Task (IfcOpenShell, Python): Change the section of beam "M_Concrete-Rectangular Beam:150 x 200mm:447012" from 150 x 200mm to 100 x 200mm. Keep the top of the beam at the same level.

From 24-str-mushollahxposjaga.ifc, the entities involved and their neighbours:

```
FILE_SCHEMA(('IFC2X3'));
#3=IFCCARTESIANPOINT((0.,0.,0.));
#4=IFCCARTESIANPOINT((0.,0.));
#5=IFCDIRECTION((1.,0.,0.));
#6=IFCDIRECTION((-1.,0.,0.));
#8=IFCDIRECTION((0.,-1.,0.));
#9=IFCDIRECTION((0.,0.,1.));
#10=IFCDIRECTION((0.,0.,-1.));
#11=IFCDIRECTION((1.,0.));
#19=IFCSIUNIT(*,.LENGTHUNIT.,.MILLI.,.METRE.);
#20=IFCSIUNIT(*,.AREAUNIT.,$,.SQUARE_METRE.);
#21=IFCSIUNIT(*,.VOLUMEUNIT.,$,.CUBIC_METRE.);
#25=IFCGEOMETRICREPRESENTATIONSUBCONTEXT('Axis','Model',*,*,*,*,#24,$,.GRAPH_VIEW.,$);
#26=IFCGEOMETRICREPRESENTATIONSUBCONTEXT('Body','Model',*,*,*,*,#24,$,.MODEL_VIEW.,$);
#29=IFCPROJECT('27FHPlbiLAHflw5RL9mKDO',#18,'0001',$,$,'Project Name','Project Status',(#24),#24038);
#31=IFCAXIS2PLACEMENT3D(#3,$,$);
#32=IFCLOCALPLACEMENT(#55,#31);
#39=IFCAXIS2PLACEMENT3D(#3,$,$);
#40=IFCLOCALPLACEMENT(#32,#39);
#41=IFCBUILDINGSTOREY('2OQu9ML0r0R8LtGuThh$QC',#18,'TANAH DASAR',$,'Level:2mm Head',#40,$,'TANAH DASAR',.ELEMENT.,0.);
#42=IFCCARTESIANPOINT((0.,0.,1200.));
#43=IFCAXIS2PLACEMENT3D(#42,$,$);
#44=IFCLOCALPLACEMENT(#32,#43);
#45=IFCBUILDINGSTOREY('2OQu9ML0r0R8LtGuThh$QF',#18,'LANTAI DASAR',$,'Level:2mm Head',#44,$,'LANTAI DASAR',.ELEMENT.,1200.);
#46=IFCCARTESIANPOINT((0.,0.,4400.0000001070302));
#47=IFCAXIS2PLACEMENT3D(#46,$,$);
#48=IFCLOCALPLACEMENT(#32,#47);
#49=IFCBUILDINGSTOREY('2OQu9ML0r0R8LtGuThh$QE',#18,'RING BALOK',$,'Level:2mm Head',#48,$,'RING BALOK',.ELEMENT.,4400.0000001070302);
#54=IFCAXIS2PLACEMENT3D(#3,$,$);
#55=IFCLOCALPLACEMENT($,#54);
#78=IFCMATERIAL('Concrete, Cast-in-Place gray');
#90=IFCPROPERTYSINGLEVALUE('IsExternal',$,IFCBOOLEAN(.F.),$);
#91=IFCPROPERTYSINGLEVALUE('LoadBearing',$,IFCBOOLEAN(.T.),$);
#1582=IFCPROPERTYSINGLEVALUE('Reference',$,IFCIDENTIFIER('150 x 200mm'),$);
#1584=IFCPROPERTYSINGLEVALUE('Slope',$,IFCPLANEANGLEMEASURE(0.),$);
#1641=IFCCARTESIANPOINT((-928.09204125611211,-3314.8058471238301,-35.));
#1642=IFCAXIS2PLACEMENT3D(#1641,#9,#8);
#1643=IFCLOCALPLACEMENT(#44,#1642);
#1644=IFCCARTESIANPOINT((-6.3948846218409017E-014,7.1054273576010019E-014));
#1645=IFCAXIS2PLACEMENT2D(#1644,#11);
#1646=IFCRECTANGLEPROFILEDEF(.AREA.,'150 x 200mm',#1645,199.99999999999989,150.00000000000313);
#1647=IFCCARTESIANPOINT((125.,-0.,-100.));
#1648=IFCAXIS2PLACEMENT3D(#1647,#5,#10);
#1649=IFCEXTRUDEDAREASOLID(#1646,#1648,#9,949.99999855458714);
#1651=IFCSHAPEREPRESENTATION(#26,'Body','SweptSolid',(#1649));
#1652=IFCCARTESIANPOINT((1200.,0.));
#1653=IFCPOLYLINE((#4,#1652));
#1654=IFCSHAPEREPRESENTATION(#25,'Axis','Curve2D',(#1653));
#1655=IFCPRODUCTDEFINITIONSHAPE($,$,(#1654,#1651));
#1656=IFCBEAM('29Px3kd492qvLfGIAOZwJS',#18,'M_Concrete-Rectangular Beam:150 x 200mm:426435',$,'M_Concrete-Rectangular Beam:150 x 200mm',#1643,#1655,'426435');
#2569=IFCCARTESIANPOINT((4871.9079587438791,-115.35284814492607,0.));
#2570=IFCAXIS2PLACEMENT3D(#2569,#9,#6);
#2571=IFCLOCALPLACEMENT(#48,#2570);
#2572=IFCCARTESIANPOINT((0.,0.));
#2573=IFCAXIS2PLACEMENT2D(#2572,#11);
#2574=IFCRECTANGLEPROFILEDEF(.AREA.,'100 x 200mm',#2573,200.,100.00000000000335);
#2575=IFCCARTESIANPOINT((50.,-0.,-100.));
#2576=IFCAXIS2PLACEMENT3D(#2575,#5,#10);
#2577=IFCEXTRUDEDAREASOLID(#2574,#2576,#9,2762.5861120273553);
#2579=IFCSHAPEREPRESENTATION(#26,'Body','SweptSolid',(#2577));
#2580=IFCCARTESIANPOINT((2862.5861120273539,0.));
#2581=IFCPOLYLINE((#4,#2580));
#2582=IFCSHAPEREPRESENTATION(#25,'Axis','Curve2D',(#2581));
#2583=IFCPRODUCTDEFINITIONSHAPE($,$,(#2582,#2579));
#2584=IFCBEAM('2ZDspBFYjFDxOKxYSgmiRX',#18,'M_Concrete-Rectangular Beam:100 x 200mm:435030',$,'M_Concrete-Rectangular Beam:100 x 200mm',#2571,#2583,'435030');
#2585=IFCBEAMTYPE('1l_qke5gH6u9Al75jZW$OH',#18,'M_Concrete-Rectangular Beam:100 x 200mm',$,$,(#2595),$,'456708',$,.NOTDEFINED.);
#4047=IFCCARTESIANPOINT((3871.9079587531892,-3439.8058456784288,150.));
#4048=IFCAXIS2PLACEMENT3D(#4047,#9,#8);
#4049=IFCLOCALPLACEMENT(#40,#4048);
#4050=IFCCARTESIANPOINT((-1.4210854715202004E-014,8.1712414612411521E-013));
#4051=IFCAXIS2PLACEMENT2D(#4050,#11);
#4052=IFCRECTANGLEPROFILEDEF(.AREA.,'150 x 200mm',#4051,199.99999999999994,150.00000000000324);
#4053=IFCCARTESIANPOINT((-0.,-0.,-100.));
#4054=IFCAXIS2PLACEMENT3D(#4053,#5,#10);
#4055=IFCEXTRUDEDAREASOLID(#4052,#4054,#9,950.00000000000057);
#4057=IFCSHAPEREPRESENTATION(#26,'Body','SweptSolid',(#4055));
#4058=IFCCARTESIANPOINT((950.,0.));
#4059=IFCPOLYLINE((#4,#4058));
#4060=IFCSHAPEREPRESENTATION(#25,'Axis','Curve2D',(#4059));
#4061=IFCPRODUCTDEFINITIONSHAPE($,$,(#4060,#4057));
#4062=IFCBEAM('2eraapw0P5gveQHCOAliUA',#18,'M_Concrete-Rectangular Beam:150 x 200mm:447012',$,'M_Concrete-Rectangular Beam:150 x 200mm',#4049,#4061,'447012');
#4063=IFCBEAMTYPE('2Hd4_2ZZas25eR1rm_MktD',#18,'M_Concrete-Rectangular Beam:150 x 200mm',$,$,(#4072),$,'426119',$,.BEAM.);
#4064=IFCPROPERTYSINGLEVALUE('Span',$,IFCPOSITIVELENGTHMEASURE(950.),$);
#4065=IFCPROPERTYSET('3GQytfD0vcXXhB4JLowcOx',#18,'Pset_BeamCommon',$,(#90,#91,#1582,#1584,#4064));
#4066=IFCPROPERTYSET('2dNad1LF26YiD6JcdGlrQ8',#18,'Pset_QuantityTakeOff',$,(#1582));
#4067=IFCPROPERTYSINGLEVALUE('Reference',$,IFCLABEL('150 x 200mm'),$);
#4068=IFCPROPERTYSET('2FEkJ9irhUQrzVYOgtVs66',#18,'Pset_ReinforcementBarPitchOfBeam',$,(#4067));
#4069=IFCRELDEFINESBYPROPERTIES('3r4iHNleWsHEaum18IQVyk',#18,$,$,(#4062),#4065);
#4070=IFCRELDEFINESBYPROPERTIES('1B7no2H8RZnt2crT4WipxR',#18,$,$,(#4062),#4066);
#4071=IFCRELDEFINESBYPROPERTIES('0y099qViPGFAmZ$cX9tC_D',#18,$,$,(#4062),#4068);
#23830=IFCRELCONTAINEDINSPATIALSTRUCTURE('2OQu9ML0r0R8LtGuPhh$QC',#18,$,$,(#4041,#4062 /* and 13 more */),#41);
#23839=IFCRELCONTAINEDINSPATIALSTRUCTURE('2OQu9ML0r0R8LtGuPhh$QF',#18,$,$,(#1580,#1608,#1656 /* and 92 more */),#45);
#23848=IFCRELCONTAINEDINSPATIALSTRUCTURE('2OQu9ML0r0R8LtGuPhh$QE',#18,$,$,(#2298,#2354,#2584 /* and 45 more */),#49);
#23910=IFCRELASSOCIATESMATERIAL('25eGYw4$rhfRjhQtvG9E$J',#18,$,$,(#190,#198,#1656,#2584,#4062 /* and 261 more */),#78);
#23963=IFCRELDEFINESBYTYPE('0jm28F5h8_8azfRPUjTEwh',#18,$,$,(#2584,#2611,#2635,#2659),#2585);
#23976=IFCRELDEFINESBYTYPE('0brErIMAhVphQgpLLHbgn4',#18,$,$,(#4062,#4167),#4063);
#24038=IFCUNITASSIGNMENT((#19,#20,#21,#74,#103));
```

```python
import ifcopenshell
import ifcopenshell.api.pset
import ifcopenshell.api.type
import ifcopenshell.util.element
import ifcopenshell.util.representation

model = ifcopenshell.open("24-str-mushollahxposjaga.ifc")

member = model.by_guid("2eraapw0P5gveQHCOAliUA")
source = next(p for p in model.by_type("IfcRectangleProfileDef") if p.ProfileName == "100 x 200mm")

body = ifcopenshell.util.representation.get_representation(member, "Model", "Body")
solid = body.Items[0]
old_profile = solid.SweptArea

# Copy the section's sizes but keep this member's own profile position.
profile = ifcopenshell.util.element.copy(model, source)
# Profiles are centred, so shift by half the change in depth to hold the top.
shift = (old_profile.XDim - profile.XDim) / 2
x, y = old_profile.Position.Location.Coordinates
up = (-1.0, 0.0)  # upwards, in the solid's own plane
location = model.createIfcCartesianPoint((x + up[0] * shift, y + up[1] * shift))
profile.Position = model.createIfcAxis2Placement2D(location, old_profile.Position.RefDirection)
solid.SweptArea = profile
if not model.get_total_inverses(old_profile):
    ifcopenshell.util.element.remove_deep2(model, old_profile)

new_type = model.by_guid("1l_qke5gH6u9Al75jZW$OH")
ifcopenshell.api.type.assign_type(
    model, related_objects=[member], relating_type=new_type, should_map_representations=False
)
member.Name = member.Name.replace("150 x 200mm", "100 x 200mm")
member.ObjectType = "M_Concrete-Rectangular Beam:100 x 200mm"
pset = model.by_id(ifcopenshell.util.element.get_pset(member, "Pset_BeamCommon", should_inherit=False)["id"])
ifcopenshell.api.pset.edit_pset(model, pset=pset, properties={"Reference": "100 x 200mm"})
pset = model.by_id(ifcopenshell.util.element.get_pset(member, "Pset_QuantityTakeOff", should_inherit=False)["id"])
ifcopenshell.api.pset.edit_pset(model, pset=pset, properties={"Reference": "100 x 200mm"})
pset = model.by_id(ifcopenshell.util.element.get_pset(member, "Pset_ReinforcementBarPitchOfBeam", should_inherit=False)["id"])
ifcopenshell.api.pset.edit_pset(model, pset=pset, properties={"Reference": "100 x 200mm"})

print(solid.SweptArea)

model.write("24-str-mushollahxposjaga_v2.ifc")
```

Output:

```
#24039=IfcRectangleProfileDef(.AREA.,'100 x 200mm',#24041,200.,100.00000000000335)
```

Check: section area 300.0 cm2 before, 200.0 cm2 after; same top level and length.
